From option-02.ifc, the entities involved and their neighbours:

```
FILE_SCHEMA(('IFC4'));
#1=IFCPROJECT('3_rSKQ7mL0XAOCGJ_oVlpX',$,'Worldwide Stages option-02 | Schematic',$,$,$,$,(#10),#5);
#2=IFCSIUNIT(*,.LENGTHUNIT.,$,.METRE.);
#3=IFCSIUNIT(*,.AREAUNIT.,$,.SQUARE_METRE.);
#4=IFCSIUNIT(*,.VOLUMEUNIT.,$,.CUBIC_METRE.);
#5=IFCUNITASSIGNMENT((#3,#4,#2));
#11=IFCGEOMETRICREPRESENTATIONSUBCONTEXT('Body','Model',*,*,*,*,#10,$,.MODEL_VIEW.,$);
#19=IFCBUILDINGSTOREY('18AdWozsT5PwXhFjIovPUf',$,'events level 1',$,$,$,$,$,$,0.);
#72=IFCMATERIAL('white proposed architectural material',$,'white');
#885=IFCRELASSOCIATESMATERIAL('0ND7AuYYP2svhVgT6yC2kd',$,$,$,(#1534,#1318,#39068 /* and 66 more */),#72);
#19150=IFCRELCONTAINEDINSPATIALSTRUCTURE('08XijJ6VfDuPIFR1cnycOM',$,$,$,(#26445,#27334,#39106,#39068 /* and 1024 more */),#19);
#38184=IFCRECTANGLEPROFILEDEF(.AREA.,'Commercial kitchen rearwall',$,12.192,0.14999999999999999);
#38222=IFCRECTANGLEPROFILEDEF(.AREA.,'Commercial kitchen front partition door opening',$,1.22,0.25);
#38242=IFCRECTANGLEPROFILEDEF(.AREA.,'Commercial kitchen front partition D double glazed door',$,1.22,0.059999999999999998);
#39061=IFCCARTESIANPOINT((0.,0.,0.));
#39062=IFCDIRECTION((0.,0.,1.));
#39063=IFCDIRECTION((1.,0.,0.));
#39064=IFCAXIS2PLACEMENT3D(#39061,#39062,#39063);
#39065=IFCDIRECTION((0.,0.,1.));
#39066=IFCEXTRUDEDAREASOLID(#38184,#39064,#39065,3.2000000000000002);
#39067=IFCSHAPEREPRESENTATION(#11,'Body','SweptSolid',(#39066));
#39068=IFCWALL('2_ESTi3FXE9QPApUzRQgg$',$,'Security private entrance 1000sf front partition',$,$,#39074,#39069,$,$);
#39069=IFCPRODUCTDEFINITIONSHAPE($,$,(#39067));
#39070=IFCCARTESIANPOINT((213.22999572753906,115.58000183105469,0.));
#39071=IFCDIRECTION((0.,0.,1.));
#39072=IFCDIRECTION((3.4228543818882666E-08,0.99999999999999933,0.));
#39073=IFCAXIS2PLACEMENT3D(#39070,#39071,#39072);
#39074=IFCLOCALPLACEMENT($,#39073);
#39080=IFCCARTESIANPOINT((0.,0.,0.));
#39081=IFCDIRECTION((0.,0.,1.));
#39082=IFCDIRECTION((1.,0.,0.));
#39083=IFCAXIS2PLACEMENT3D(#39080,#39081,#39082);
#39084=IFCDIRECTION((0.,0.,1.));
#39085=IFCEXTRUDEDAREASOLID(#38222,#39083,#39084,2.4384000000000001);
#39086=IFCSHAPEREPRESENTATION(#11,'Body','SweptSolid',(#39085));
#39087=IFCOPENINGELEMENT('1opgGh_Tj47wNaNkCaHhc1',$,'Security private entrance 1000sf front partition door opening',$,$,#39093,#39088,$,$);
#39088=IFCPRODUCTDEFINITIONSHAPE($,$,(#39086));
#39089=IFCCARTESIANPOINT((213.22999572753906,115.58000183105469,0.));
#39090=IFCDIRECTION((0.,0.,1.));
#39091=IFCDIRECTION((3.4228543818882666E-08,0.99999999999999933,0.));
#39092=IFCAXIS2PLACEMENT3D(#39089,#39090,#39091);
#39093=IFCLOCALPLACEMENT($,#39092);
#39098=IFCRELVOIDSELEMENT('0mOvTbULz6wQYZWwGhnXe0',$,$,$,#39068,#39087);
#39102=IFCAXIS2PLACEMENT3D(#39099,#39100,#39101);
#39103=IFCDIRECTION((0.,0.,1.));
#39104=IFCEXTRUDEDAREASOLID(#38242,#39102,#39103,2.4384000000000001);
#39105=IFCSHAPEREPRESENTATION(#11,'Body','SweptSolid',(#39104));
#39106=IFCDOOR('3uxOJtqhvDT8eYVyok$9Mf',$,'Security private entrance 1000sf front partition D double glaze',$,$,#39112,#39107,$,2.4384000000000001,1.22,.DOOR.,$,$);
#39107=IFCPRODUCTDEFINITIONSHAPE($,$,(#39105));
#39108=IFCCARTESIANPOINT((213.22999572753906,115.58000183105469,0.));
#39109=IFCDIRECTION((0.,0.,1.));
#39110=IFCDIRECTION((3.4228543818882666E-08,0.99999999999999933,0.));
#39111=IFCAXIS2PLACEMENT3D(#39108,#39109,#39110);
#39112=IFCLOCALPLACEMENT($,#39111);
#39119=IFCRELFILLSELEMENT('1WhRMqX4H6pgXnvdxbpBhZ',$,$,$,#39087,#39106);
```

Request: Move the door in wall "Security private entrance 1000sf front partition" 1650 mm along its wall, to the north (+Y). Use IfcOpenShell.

```python
import ifcopenshell
import ifcopenshell.api.geometry
import ifcopenshell.util.placement

model = ifcopenshell.open("option-02.ifc")

door = model.by_id(39106)
opening = door.FillsVoids[0].RelatingOpeningElement
wall = opening.VoidsElements[0].RelatingBuildingElement

wall_matrix = ifcopenshell.util.placement.get_local_placement(wall.ObjectPlacement)
shift = wall_matrix[:3, 0] * 1.65
before = ifcopenshell.util.placement.get_local_placement(door.ObjectPlacement)[:3, 3].copy()

# The door is not placed relative to its opening, so move both.
for product in (opening, door):
    matrix = ifcopenshell.util.placement.get_local_placement(product.ObjectPlacement)
    matrix[:3, 3] += shift
    ifcopenshell.api.geometry.edit_object_placement(model, product=product, matrix=matrix, is_si=False)

after = ifcopenshell.util.placement.get_local_placement(door.ObjectPlacement)[:3, 3]
print("door moved by", (after - before).round(3) + 0.0)

model.write("option-02-out.ifc")
```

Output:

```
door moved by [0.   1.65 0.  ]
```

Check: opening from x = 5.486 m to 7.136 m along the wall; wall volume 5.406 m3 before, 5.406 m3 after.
